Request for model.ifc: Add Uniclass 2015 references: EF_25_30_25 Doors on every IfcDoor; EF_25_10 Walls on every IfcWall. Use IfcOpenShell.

First a look at what the model holds.

```python
import ifcopenshell

model = ifcopenshell.open("model.ifc")
print(model.schema)
print("classifications:", [c.Name for c in model.by_type("IfcClassification")])
for ifc_class in ("IfcDoor", "IfcRoof", "IfcStair", "IfcWall", "IfcWindow"):
    print(ifc_class, len(model.by_type(ifc_class)))
```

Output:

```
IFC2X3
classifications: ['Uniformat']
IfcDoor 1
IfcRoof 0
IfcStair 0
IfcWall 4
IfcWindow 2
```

```python
import ifcopenshell
import ifcopenshell.api.classification

model = ifcopenshell.open("model.ifc")

# IFC2X3 requires Source and Edition and has no link from the project to the system.
system = model.create_entity("IfcClassification", Source="NBS", Edition="2015", Name="Uniclass 2015")

codes = {
    "IfcDoor": ("EF_25_30_25", "Doors"),
    "IfcWall": ("EF_25_10", "Walls"),
}
for ifc_class, (code, name) in codes.items():
    products = model.by_type(ifc_class)
    ifcopenshell.api.classification.add_reference(
        model, products=products, classification=system, identification=code, name=name
    )
    print(code, len(products))

model.write("model_rev.ifc")
```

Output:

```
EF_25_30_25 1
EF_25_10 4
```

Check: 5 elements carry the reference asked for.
